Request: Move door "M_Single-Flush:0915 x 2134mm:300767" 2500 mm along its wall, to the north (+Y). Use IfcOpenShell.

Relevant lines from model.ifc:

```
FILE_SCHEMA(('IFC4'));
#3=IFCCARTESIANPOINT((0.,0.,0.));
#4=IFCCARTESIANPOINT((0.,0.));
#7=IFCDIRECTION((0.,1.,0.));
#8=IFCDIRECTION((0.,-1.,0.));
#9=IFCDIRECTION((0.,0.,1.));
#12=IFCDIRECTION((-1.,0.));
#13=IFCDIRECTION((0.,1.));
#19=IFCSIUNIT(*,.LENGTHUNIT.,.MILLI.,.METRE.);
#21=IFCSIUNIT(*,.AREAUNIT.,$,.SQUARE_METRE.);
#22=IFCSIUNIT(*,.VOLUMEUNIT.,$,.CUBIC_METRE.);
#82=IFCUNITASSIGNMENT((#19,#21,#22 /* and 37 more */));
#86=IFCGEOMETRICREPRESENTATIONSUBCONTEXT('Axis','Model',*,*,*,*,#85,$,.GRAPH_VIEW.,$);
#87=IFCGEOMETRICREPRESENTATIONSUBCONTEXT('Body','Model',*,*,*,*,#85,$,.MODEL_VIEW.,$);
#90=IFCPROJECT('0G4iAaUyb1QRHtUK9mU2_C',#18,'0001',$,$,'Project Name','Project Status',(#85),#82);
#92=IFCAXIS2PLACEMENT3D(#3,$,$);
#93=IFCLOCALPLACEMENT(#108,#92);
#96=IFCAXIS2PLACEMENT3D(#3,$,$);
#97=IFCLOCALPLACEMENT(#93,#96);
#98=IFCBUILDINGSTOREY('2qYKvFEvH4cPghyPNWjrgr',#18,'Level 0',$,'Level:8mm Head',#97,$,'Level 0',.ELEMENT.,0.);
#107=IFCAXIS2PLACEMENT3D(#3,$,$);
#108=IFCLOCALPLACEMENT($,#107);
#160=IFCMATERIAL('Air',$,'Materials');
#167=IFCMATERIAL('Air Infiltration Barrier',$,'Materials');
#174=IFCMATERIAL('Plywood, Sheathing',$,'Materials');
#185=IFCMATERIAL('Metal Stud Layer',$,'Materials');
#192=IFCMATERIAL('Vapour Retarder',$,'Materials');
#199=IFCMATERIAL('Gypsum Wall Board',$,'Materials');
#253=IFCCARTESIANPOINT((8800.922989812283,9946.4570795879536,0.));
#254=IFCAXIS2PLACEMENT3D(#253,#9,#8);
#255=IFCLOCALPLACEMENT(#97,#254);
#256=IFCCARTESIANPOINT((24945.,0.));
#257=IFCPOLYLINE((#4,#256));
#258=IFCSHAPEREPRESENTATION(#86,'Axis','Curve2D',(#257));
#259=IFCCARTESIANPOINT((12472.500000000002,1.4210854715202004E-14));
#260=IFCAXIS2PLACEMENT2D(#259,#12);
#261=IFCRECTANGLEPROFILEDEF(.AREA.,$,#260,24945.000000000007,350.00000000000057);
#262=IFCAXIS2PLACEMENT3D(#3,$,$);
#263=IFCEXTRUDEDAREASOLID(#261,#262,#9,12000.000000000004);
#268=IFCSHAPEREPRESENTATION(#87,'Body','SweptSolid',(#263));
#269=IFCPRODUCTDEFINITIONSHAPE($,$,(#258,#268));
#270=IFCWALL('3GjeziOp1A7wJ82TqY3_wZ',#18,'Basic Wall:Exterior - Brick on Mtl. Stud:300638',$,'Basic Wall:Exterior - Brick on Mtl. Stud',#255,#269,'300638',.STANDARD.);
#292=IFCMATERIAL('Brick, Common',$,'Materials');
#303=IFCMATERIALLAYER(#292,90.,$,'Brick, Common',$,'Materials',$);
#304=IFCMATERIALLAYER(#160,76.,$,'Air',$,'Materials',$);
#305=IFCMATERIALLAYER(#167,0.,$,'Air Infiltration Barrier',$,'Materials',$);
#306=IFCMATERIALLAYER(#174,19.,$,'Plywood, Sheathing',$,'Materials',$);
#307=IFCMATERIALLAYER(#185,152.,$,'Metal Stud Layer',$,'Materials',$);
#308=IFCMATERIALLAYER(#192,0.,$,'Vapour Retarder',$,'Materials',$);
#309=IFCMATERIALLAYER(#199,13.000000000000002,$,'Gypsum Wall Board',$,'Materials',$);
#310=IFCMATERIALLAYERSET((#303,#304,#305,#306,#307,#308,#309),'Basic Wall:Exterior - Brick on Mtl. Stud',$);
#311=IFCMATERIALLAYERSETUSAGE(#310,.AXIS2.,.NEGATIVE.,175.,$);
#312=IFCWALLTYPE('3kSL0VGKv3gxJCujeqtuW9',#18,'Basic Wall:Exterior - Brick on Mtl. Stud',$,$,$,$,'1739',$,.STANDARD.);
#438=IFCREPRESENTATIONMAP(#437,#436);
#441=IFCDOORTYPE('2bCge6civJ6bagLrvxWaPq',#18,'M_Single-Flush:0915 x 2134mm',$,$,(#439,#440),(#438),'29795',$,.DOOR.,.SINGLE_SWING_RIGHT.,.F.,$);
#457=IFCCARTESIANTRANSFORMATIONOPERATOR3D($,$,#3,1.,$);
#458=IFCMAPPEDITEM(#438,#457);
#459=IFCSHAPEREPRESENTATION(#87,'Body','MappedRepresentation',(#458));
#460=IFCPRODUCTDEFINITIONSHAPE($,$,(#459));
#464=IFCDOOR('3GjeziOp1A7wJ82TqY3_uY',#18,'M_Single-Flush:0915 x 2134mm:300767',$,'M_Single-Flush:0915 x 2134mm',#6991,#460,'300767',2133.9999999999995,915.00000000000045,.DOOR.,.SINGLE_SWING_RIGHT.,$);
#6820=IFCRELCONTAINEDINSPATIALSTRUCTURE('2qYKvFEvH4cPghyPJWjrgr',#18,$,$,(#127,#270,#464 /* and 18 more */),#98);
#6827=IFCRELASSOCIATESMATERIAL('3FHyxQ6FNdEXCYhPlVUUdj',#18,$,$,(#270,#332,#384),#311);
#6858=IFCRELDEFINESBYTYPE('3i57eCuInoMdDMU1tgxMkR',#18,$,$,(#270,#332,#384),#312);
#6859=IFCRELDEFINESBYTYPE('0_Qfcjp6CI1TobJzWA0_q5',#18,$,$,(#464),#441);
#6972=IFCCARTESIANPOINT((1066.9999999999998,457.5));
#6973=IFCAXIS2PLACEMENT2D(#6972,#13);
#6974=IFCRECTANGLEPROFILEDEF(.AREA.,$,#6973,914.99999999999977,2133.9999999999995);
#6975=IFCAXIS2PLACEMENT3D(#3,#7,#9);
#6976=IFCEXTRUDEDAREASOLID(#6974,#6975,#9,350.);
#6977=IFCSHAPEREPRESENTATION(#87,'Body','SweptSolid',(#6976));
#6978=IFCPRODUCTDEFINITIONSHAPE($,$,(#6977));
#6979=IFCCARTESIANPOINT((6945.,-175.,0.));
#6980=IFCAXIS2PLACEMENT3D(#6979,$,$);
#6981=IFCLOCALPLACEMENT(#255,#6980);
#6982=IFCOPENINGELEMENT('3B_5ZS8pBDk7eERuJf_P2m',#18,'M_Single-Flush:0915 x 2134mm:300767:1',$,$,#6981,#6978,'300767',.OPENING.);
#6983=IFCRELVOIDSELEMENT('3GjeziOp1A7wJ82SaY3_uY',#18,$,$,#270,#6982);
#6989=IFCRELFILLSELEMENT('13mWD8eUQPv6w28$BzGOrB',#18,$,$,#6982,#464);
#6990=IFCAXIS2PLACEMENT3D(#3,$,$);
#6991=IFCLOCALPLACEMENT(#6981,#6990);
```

```python
import ifcopenshell
import ifcopenshell.api.geometry
import ifcopenshell.util.placement
import ifcopenshell.util.unit

model = ifcopenshell.open("model.ifc")
unit_scale = ifcopenshell.util.unit.calculate_unit_scale(model)

door = model.by_id(464)
opening = door.FillsVoids[0].RelatingOpeningElement
wall = opening.VoidsElements[0].RelatingBuildingElement

wall_matrix = ifcopenshell.util.placement.get_local_placement(wall.ObjectPlacement)
shift = wall_matrix[:3, 0] * -2.5 / unit_scale
before = ifcopenshell.util.placement.get_local_placement(door.ObjectPlacement)[:3, 3].copy()

# The door is placed relative to its opening, so it follows when the opening moves.
matrix = ifcopenshell.util.placement.get_local_placement(opening.ObjectPlacement)
matrix[:3, 3] += shift
ifcopenshell.api.geometry.edit_object_placement(
    model, product=opening, matrix=matrix, is_si=False, should_transform_children=True
)

after = ifcopenshell.util.placement.get_local_placement(door.ObjectPlacement)[:3, 3]
print("door moved by", (after - before).round(3) + 0.0)

model.write("model_v2.ifc")
```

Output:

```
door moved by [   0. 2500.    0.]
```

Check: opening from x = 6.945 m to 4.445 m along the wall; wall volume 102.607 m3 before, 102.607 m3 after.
